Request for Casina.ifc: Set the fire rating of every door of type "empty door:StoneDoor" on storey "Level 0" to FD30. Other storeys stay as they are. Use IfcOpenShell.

First a look at what the model holds.

```python
import ifcopenshell
import ifcopenshell.util.element

model = ifcopenshell.open("Casina.ifc")
print(model.schema)
storey = next(s for s in model.by_type("IfcBuildingStorey") if s.Name == "Level 0")
doors = [e for e in ifcopenshell.util.element.get_decomposition(storey) if e.is_a("IfcDoor")]
seen = {}
for e in doors:
    element_type = ifcopenshell.util.element.get_type(e)
    key = (element_type.Name if element_type != e and element_type else None, ifcopenshell.util.element.get_pset(e, "Pset_DoorCommon", "FireRating"))
    seen[key] = seen.get(key, 0) + 1
for (name, value), count in sorted(seen.items(), key=str):
    print(count, "x", name, "|", value)
```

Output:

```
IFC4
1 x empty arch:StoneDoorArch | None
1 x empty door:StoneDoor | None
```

```python
import ifcopenshell
import ifcopenshell.api.pset
import ifcopenshell.util.element

model = ifcopenshell.open("Casina.ifc")

storey = next(s for s in model.by_type("IfcBuildingStorey") if s.Name == "Level 0")
doors = [e for e in ifcopenshell.util.element.get_decomposition(storey) if e.is_a("IfcDoor")]

count = 0
for e in doors:
    element_type = ifcopenshell.util.element.get_type(e)
    if element_type in (None, e) or element_type.Name != "empty door:StoneDoor":
        continue
    # add_pset returns the element's existing set when there is one.
    pset = ifcopenshell.api.pset.add_pset(model, product=e, name="Pset_DoorCommon")
    ifcopenshell.api.pset.edit_pset(model, pset=pset, properties={"FireRating": "FD30"})
    count += 1

print(count, "doors updated")

model.write("Casina_v2.ifc")
```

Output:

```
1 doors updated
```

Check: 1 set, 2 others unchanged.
